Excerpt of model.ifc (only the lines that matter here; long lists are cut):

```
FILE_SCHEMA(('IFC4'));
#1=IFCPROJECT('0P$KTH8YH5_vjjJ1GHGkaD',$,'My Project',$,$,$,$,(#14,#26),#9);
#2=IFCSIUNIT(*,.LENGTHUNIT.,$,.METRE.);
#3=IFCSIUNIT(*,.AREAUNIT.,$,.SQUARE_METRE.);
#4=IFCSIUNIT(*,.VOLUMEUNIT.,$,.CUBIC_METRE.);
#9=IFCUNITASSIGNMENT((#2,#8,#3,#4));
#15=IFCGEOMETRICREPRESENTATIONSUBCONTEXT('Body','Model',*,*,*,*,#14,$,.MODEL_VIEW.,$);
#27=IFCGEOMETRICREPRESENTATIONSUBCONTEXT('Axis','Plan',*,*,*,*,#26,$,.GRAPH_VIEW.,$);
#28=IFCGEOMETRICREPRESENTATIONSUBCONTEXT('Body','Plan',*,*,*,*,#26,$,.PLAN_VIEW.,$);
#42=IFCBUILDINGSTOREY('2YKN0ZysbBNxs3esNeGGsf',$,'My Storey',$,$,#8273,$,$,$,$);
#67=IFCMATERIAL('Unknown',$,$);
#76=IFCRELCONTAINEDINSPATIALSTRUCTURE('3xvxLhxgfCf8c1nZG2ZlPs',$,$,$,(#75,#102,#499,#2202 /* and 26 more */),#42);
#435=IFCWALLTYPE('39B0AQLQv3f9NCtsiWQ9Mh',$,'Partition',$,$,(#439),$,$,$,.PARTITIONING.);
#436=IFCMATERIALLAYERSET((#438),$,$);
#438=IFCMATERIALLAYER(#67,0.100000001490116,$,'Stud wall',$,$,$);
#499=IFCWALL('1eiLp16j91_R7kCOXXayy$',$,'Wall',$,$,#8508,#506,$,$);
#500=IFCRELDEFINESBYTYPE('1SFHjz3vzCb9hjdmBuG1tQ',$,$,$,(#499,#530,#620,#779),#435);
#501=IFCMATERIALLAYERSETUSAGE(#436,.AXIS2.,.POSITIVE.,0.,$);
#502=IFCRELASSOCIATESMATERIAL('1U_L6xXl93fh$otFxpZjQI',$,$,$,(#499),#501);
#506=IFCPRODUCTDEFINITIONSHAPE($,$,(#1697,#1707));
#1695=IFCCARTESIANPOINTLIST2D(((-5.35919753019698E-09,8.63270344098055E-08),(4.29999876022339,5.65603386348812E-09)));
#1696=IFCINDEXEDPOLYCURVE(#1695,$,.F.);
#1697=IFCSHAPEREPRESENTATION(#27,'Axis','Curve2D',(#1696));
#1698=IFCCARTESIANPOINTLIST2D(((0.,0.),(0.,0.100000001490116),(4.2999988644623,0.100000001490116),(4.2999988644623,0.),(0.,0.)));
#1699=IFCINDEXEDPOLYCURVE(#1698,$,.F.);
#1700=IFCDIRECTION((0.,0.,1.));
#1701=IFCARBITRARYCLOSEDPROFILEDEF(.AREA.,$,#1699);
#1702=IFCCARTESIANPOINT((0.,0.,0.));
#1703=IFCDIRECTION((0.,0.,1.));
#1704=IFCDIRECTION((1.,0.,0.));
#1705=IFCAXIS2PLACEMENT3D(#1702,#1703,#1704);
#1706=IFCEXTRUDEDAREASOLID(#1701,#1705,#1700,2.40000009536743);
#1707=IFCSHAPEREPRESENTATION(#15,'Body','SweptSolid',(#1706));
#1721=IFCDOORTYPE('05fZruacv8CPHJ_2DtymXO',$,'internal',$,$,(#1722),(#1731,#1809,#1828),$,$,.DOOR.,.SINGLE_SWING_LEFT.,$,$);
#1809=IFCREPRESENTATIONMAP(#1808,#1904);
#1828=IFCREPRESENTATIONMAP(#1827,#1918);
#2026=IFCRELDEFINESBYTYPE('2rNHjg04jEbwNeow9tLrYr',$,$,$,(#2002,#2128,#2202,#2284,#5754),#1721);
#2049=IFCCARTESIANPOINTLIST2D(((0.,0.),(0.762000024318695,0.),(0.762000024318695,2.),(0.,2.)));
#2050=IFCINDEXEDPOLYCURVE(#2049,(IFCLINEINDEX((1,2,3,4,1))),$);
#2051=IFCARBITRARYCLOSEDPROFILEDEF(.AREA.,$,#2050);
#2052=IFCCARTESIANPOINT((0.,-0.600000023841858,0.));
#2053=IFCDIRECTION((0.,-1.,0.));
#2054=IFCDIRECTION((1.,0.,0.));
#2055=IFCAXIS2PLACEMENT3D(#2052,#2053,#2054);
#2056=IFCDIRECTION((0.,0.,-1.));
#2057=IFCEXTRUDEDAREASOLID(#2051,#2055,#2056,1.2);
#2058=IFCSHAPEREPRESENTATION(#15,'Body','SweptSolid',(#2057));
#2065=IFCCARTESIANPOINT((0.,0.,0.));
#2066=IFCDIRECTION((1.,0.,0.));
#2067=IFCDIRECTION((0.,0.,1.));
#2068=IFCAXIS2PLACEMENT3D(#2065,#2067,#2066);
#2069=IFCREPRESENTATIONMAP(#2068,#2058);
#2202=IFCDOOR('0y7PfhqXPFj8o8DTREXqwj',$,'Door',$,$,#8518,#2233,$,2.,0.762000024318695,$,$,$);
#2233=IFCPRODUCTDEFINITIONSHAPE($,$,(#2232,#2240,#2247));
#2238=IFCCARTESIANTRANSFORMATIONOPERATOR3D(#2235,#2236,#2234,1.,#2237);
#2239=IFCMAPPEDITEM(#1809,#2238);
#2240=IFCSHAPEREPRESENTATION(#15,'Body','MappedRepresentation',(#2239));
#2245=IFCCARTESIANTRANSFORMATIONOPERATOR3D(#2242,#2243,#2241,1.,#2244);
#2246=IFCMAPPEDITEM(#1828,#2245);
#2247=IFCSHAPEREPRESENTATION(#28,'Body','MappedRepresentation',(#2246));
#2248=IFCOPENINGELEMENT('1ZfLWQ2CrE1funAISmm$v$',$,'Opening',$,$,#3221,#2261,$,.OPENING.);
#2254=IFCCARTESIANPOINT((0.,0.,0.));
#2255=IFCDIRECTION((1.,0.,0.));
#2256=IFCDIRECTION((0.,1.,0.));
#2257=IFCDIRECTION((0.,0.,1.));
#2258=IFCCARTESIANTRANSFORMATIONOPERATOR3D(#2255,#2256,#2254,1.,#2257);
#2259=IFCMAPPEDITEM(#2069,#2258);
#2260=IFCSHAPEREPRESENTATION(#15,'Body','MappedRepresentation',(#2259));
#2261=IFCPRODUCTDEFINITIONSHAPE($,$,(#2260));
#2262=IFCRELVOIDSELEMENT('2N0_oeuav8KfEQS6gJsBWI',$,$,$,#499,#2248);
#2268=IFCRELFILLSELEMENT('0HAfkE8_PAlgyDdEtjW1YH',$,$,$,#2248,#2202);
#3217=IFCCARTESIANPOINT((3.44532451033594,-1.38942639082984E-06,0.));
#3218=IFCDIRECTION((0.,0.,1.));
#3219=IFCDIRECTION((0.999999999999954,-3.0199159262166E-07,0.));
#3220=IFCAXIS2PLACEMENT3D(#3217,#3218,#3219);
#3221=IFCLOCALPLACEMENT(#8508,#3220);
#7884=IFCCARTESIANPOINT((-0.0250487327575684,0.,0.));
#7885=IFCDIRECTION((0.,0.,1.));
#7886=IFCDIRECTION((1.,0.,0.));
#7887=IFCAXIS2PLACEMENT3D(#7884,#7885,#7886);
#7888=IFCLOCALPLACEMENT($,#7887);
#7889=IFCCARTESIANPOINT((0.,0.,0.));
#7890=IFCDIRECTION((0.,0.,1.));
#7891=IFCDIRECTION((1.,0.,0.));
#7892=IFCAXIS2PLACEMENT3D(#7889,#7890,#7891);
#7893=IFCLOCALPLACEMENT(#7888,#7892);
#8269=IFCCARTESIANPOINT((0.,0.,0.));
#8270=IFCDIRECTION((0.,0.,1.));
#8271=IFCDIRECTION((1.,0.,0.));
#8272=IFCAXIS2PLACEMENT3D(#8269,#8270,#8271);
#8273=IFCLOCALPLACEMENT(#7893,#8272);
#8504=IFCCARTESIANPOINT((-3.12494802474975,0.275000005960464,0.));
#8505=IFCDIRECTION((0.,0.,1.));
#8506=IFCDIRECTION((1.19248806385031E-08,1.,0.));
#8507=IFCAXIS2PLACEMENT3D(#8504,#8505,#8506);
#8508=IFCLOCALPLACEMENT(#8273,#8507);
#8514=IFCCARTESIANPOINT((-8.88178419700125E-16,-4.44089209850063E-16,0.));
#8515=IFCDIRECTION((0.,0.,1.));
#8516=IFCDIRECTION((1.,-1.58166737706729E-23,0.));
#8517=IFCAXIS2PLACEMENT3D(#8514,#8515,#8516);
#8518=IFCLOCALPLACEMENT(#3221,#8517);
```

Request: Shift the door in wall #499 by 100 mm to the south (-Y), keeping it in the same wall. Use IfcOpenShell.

```python
import ifcopenshell
import ifcopenshell.api.geometry
import ifcopenshell.util.placement
import ifcopenshell.util.unit

model = ifcopenshell.open("model.ifc")
unit_scale = ifcopenshell.util.unit.calculate_unit_scale(model)

door = model.by_guid("0y7PfhqXPFj8o8DTREXqwj")
opening = door.FillsVoids[0].RelatingOpeningElement
wall = opening.VoidsElements[0].RelatingBuildingElement

wall_matrix = ifcopenshell.util.placement.get_local_placement(wall.ObjectPlacement)
shift = wall_matrix[:3, 0] * -0.1 / unit_scale
before = ifcopenshell.util.placement.get_local_placement(door.ObjectPlacement)[:3, 3].copy()

# The door is placed relative to its opening, so it follows when the opening moves.
matrix = ifcopenshell.util.placement.get_local_placement(opening.ObjectPlacement)
matrix[:3, 3] += shift
ifcopenshell.api.geometry.edit_object_placement(
    model, product=opening, matrix=matrix, is_si=False, should_transform_children=True
)

after = ifcopenshell.util.placement.get_local_placement(door.ObjectPlacement)[:3, 3]
print("door moved by", (after - before).round(3) + 0.0)

model.write("model_updated.ifc")
```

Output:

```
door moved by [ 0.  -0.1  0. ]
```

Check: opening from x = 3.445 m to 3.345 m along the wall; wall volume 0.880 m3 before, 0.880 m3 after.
